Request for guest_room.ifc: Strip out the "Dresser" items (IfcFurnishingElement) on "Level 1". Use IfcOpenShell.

First a look at what the model holds.

```python
import ifcopenshell
import ifcopenshell.util.element

model = ifcopenshell.open("guest_room.ifc")
print(model.schema)
storey = next(s for s in model.by_type("IfcBuildingStorey") if s.Name == "Level 1")
furniture = [e for e in ifcopenshell.util.element.get_decomposition(storey) if e.is_a("IfcFurnishingElement")]
seen = {}
for e in furniture:
    element_type = ifcopenshell.util.element.get_type(e)
    name = element_type.Name if element_type not in (None, e) else None
    seen[name] = seen.get(name, 0) + 1
for name, count in sorted(seen.items(), key=str):
    print(count, "x", name)
```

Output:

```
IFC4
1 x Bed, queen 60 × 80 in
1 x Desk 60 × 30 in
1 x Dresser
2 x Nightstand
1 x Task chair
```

```python
import ifcopenshell
import ifcopenshell.api.root
import ifcopenshell.util.element

model = ifcopenshell.open("guest_room.ifc")

storey = next(s for s in model.by_type("IfcBuildingStorey") if s.Name == "Level 1")
furniture = [e for e in ifcopenshell.util.element.get_decomposition(storey) if e.is_a("IfcFurnishingElement")]
targets = [e for e in furniture if (t := ifcopenshell.util.element.get_type(e)) not in (None, e) and t.Name == "Dresser"]

for e in targets:
    ifcopenshell.api.root.remove_product(model, product=e)
print(len(targets), "removed")

model.write("guest_room_edited.ifc")
```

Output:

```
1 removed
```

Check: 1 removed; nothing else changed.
